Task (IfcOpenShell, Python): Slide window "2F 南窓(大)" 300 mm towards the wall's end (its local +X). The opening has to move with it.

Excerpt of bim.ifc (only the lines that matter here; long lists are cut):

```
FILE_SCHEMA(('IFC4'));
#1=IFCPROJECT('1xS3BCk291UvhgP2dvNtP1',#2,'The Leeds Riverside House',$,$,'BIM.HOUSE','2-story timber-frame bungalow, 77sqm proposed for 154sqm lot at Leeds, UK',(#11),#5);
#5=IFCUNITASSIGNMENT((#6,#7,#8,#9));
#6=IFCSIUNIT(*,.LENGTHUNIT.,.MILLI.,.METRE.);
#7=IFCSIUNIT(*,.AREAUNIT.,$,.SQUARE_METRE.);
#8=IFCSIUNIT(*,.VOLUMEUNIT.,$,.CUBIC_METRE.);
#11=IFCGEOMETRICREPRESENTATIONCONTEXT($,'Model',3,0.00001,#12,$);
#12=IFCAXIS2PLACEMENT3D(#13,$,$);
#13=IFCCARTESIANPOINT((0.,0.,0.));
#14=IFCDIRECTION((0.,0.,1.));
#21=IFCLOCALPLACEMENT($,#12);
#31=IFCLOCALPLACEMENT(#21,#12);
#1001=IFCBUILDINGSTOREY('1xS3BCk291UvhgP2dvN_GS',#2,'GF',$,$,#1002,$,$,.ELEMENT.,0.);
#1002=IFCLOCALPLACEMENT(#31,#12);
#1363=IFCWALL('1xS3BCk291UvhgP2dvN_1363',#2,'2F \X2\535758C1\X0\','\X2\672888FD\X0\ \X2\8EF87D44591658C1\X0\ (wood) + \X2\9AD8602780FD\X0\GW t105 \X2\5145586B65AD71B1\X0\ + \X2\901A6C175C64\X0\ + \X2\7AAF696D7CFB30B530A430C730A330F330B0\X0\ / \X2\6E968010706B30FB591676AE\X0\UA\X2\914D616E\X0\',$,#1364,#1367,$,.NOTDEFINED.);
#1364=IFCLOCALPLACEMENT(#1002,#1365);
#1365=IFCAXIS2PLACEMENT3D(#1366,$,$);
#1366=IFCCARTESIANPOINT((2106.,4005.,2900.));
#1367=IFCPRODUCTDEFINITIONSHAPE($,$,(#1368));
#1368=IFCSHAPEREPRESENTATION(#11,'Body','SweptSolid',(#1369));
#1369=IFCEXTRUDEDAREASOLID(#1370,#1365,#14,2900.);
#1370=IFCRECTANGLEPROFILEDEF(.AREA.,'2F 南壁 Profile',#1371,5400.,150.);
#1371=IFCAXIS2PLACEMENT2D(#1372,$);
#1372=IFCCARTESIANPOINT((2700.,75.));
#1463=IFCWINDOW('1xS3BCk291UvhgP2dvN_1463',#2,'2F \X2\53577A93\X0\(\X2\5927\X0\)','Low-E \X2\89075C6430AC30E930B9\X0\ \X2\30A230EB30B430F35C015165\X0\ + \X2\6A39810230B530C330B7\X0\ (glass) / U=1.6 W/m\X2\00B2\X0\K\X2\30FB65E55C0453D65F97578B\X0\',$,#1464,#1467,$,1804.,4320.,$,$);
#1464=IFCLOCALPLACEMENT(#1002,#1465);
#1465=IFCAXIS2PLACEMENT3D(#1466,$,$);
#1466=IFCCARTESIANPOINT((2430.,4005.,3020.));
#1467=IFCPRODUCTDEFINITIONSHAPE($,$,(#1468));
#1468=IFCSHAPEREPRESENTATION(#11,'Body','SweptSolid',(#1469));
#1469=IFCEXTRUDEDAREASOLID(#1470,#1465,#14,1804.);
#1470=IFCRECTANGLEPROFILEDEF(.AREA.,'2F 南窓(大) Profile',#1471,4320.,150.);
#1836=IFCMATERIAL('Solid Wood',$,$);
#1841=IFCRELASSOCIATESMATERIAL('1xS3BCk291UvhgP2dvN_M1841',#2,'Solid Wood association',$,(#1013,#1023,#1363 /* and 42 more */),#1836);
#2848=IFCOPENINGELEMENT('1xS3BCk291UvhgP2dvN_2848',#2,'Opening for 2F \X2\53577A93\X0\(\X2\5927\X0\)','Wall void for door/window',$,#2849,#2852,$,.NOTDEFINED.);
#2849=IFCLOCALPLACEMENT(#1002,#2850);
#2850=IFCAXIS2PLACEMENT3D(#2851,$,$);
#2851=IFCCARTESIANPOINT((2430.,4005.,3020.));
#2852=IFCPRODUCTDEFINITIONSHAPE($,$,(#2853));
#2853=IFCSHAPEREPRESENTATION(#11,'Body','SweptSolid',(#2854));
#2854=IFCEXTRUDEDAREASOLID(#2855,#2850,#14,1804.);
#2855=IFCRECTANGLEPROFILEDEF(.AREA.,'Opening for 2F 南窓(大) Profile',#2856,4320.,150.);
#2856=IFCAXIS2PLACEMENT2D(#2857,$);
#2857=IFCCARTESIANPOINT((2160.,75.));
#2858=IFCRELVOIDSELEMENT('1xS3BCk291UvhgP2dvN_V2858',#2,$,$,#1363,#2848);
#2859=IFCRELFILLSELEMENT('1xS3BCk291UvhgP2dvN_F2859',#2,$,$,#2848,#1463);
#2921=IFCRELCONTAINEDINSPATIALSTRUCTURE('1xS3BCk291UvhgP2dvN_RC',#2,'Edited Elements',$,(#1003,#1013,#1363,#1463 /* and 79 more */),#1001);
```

```python
import ifcopenshell
import ifcopenshell.api.geometry
import ifcopenshell.util.placement
import ifcopenshell.util.unit

model = ifcopenshell.open("bim.ifc")
unit_scale = ifcopenshell.util.unit.calculate_unit_scale(model)

window = model.by_id(1463)
opening = window.FillsVoids[0].RelatingOpeningElement
wall = opening.VoidsElements[0].RelatingBuildingElement

wall_matrix = ifcopenshell.util.placement.get_local_placement(wall.ObjectPlacement)
shift = wall_matrix[:3, 0] * 0.3 / unit_scale
before = ifcopenshell.util.placement.get_local_placement(window.ObjectPlacement)[:3, 3].copy()

# The window is not placed relative to its opening, so move both.
for product in (opening, window):
    matrix = ifcopenshell.util.placement.get_local_placement(product.ObjectPlacement)
    matrix[:3, 3] += shift
    ifcopenshell.api.geometry.edit_object_placement(model, product=product, matrix=matrix, is_si=False)

after = ifcopenshell.util.placement.get_local_placement(window.ObjectPlacement)[:3, 3]
print("window moved by", (after - before).round(3) + 0.0)

model.write("bim_edited.ifc")
```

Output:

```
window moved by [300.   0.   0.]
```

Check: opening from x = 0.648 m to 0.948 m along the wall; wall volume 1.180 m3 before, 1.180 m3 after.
